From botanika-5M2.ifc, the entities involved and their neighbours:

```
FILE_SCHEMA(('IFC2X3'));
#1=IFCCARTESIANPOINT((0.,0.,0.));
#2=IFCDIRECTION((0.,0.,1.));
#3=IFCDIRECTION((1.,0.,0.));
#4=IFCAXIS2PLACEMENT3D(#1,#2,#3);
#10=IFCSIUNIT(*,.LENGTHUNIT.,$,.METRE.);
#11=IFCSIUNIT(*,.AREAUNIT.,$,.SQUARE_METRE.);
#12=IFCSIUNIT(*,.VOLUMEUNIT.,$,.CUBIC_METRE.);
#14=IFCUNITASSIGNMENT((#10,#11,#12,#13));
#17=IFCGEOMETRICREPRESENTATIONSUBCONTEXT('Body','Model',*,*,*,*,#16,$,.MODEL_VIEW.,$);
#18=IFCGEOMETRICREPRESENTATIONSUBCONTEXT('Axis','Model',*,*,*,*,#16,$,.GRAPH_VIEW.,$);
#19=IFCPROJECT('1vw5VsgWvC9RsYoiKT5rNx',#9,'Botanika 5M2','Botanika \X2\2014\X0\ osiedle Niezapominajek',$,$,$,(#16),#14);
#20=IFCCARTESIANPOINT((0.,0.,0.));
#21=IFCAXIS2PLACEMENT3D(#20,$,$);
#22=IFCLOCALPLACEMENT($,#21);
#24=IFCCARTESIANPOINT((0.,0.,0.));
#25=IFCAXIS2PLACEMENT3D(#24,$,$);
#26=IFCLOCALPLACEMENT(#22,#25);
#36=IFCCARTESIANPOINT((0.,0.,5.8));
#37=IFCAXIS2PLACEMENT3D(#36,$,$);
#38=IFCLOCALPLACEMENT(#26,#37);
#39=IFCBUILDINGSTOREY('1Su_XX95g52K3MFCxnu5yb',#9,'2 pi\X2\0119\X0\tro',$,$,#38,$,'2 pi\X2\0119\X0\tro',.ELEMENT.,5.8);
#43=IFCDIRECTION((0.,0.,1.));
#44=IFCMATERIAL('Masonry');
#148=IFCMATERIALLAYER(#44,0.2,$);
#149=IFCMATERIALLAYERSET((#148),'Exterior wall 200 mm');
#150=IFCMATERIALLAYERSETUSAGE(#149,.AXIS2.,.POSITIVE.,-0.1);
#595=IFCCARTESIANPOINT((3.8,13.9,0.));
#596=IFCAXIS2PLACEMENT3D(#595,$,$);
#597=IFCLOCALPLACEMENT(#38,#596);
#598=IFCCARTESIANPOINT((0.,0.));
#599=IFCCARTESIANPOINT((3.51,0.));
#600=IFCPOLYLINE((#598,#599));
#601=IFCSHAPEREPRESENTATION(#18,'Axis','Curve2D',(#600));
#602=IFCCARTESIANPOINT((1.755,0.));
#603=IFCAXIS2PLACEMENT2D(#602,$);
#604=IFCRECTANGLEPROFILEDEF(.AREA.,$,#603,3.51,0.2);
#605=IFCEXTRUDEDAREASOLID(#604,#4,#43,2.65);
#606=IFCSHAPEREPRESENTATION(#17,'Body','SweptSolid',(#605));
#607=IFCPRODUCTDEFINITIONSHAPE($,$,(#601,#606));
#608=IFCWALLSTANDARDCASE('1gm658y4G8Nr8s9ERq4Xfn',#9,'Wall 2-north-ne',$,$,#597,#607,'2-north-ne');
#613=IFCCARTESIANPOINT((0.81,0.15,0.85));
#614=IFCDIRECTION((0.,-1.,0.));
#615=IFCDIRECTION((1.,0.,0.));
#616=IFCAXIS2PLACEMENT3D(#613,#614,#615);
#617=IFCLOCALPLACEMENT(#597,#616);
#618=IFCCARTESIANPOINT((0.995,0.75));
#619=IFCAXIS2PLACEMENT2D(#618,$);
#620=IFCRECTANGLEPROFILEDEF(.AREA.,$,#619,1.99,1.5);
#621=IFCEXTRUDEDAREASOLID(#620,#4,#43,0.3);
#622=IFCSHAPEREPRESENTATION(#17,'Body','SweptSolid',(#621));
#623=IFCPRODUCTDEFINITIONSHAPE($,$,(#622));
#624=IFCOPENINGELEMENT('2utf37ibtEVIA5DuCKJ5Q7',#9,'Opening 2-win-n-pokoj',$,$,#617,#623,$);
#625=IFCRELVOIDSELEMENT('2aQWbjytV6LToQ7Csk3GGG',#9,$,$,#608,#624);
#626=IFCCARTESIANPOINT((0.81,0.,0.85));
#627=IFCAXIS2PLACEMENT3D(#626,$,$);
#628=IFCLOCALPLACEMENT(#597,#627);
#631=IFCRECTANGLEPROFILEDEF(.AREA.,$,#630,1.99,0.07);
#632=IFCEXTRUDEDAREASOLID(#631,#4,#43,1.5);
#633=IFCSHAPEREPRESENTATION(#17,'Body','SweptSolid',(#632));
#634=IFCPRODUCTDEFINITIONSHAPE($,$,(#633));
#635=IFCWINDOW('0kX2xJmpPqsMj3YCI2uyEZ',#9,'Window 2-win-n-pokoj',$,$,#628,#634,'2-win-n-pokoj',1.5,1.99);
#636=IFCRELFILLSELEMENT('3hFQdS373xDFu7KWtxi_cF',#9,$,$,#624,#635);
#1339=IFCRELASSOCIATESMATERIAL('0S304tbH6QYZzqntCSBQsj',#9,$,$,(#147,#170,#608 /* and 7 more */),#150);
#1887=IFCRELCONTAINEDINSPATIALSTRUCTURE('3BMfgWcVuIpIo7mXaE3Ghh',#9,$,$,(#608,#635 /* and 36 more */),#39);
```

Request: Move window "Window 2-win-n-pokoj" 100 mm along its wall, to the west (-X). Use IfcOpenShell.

```python
import ifcopenshell
import ifcopenshell.api.geometry
import ifcopenshell.util.placement

model = ifcopenshell.open("botanika-5M2.ifc")

window = model.by_guid("0kX2xJmpPqsMj3YCI2uyEZ")
opening = window.FillsVoids[0].RelatingOpeningElement
wall = opening.VoidsElements[0].RelatingBuildingElement

wall_matrix = ifcopenshell.util.placement.get_local_placement(wall.ObjectPlacement)
shift = wall_matrix[:3, 0] * -0.1
before = ifcopenshell.util.placement.get_local_placement(window.ObjectPlacement)[:3, 3].copy()

# The window is not placed relative to its opening, so move both.
for product in (opening, window):
    matrix = ifcopenshell.util.placement.get_local_placement(product.ObjectPlacement)
    matrix[:3, 3] += shift
    ifcopenshell.api.geometry.edit_object_placement(model, product=product, matrix=matrix, is_si=False)

after = ifcopenshell.util.placement.get_local_placement(window.ObjectPlacement)[:3, 3]
print("window moved by", (after - before).round(3) + 0.0)

model.write("botanika-5M2_rev.ifc")
```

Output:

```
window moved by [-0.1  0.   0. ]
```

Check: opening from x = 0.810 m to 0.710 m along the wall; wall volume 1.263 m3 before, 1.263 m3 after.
